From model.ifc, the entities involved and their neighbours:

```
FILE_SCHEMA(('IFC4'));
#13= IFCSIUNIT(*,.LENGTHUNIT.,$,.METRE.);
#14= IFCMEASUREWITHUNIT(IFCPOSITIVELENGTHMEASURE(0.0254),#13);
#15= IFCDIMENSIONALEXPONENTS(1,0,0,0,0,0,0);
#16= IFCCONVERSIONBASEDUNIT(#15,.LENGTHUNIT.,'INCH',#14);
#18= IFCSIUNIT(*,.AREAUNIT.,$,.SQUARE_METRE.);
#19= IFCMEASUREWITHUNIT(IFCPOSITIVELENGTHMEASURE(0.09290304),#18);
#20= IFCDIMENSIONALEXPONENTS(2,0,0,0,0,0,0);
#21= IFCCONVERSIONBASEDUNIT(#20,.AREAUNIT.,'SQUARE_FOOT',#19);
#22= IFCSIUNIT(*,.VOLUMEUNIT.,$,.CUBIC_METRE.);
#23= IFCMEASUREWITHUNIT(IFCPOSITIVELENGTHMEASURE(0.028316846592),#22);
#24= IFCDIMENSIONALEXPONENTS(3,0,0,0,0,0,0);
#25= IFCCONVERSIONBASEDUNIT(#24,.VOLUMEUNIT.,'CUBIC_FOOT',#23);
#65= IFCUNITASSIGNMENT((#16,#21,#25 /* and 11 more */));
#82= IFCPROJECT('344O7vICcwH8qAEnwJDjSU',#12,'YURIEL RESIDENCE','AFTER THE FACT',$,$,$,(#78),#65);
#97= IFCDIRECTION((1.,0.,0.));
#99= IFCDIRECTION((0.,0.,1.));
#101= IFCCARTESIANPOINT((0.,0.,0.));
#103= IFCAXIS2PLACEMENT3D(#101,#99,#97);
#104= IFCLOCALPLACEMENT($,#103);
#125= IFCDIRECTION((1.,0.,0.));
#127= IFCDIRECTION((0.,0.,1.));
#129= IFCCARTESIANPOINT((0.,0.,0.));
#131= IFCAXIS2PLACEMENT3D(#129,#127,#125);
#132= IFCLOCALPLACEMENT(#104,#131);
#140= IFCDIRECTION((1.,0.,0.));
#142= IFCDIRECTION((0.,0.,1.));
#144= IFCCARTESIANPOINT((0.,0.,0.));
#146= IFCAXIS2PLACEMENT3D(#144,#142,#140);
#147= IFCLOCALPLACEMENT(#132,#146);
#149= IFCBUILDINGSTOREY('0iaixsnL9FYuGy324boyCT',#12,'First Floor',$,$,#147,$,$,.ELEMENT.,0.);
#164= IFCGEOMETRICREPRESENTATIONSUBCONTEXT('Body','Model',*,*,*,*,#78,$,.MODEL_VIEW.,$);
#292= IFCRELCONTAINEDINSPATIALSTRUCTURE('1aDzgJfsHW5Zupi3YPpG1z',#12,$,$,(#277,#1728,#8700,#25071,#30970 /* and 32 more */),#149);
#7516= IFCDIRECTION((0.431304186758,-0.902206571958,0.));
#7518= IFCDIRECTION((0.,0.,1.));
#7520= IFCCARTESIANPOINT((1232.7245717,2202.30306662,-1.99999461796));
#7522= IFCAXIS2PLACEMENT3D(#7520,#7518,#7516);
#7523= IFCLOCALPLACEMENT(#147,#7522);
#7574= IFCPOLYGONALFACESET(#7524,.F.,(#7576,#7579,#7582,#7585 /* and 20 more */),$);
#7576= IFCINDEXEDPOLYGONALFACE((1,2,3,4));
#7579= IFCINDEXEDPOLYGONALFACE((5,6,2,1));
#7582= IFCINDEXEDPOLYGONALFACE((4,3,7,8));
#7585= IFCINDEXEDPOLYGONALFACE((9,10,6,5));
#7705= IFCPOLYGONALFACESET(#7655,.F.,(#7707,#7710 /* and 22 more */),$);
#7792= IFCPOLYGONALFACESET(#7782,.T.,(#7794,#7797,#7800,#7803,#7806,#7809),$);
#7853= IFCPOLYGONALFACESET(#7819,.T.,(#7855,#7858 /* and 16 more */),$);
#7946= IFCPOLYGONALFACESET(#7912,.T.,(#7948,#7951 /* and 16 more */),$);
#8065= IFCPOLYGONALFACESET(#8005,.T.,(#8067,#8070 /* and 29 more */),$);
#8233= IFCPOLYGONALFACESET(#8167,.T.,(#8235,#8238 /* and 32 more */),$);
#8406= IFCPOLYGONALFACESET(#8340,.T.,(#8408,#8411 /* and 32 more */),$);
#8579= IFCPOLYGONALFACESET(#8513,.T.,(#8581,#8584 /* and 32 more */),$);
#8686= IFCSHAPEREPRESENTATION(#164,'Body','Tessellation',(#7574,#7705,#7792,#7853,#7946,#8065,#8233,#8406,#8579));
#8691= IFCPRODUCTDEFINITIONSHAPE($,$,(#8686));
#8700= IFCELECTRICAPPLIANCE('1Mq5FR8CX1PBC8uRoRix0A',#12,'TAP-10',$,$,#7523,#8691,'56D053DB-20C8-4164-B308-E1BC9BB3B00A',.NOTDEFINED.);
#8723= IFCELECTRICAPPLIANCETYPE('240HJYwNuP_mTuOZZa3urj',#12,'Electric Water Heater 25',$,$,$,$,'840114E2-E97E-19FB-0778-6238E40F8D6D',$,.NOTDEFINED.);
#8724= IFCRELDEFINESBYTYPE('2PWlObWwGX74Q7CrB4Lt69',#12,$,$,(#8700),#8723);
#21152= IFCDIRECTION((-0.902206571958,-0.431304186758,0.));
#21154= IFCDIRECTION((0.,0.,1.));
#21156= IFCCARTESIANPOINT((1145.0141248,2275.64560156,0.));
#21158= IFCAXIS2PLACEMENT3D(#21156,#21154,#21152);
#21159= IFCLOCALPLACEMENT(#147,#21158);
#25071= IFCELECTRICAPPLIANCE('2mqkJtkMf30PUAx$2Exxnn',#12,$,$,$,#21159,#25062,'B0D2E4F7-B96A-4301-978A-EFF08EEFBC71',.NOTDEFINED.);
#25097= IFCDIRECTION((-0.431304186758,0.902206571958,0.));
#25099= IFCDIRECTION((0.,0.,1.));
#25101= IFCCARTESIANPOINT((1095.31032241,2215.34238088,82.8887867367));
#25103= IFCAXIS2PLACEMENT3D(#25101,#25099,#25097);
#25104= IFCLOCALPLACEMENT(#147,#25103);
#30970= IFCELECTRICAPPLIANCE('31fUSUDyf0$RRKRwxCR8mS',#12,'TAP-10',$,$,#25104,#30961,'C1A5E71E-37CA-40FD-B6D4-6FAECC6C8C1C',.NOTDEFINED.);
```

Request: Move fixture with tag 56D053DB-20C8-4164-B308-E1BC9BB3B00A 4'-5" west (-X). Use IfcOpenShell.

```python
import ifcopenshell
import ifcopenshell.api.geometry
import ifcopenshell.util.placement
import ifcopenshell.util.unit

model = ifcopenshell.open("model.ifc")
unit_scale = ifcopenshell.util.unit.calculate_unit_scale(model)

item = model.by_id(8700)
matrix = ifcopenshell.util.placement.get_local_placement(item.ObjectPlacement)
matrix[0, 3] -= 53 * 0.0254 / unit_scale
ifcopenshell.api.geometry.edit_object_placement(model, product=item, matrix=matrix, is_si=False)

print(ifcopenshell.util.placement.get_local_placement(item.ObjectPlacement).round(3) + 0.0)

model.write("model-out.ifc")
```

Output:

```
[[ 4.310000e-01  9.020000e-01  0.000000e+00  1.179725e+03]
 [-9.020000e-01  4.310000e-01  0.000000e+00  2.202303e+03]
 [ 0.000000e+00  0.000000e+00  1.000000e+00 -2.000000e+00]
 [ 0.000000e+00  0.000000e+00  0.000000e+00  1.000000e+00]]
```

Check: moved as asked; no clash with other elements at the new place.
